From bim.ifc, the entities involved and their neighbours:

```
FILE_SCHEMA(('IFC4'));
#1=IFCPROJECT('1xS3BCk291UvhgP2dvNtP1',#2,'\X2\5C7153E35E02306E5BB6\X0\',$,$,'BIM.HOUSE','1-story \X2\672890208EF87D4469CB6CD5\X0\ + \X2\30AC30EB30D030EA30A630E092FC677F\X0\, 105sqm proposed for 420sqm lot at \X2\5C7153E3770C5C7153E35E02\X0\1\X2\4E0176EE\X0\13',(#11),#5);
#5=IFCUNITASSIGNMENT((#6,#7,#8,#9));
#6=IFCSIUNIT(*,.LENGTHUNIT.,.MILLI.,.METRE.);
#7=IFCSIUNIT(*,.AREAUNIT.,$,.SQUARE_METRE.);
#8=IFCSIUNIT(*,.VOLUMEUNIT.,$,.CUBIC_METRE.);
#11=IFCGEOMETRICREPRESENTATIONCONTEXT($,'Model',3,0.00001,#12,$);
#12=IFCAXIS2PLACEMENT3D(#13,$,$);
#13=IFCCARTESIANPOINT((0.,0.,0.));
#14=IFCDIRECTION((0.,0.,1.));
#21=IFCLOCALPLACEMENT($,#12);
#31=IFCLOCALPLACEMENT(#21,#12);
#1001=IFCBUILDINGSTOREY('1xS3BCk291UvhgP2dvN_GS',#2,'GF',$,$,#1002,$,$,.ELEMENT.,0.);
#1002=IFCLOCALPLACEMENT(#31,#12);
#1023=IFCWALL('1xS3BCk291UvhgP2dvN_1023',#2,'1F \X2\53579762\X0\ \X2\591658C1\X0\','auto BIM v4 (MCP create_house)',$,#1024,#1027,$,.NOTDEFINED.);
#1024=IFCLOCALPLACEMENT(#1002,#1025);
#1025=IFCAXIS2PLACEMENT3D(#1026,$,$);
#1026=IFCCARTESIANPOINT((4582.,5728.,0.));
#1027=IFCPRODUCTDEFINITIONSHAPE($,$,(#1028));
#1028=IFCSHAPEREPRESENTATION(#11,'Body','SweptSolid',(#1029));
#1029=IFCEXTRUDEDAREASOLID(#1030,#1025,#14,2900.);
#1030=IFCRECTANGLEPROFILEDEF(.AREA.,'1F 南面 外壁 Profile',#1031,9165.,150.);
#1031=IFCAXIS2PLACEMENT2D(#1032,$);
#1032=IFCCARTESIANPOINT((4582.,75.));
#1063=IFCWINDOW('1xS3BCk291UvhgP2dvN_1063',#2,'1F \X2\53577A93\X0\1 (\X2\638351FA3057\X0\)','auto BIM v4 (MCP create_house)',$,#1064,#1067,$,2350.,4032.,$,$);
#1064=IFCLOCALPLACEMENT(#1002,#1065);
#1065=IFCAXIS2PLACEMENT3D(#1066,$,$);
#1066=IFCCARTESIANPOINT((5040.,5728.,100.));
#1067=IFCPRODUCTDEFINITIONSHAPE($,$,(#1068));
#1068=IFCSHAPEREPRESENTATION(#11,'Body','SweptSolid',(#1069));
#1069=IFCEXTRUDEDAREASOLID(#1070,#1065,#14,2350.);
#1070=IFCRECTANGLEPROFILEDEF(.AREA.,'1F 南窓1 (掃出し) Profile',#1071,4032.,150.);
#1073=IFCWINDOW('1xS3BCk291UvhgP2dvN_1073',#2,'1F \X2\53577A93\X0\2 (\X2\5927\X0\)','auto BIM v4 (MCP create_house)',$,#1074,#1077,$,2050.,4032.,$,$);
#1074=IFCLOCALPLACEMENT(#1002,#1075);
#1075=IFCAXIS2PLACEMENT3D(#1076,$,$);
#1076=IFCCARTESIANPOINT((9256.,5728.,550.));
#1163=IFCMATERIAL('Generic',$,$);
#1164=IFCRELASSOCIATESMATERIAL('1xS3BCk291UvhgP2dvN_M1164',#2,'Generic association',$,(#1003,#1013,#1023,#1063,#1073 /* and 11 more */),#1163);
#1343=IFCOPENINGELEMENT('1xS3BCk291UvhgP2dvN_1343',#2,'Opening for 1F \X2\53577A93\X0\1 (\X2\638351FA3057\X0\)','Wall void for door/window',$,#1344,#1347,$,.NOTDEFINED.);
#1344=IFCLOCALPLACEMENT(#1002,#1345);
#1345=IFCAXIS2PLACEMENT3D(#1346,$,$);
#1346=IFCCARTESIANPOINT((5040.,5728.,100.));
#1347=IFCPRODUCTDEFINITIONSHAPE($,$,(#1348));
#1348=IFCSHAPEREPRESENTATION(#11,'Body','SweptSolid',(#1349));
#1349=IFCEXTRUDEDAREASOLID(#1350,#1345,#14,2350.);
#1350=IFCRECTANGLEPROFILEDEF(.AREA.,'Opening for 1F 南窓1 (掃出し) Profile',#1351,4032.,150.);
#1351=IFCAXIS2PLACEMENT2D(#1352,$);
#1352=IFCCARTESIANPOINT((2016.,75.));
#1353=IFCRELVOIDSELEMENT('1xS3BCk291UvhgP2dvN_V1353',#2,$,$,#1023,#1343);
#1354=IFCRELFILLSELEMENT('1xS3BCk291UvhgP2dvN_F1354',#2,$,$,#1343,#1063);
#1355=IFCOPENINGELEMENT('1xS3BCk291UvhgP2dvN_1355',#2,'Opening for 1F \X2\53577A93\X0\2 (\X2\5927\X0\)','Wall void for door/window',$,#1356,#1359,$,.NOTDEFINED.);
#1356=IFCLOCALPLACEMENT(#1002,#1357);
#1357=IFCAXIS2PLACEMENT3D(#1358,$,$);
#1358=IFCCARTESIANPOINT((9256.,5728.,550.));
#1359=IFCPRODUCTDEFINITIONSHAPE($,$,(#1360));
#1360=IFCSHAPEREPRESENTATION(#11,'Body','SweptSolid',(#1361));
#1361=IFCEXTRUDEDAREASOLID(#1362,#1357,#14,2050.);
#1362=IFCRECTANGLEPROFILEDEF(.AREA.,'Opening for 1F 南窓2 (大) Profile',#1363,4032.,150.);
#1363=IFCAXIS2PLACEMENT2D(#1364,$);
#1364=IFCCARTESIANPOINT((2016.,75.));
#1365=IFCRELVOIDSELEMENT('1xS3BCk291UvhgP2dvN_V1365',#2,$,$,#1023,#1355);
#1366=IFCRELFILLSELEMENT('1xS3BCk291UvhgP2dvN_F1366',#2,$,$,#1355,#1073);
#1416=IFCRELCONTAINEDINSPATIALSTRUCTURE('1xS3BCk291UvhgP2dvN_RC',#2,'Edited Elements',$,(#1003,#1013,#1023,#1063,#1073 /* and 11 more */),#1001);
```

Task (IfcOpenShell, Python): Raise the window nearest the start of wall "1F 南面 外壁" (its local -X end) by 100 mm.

```python
import numpy as np
import ifcopenshell
import ifcopenshell.api.geometry
import ifcopenshell.util.placement
import ifcopenshell.util.unit

model = ifcopenshell.open("bim.ifc")
unit_scale = ifcopenshell.util.unit.calculate_unit_scale(model)

window = model.by_id(1063)
opening = window.FillsVoids[0].RelatingOpeningElement
dz = 0.1 / unit_scale

shift = np.array([0.0, 0.0, dz])
# The window is not placed relative to its opening, so move both.
for product in (opening, window):
    matrix = ifcopenshell.util.placement.get_local_placement(product.ObjectPlacement)
    matrix[:3, 3] += shift
    ifcopenshell.api.geometry.edit_object_placement(model, product=product, matrix=matrix, is_si=False)

print(f"moved by {dz * unit_scale:+.3f} m")

model.write("bim_v2.ifc")
```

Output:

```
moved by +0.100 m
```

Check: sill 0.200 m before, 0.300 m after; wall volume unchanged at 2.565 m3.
